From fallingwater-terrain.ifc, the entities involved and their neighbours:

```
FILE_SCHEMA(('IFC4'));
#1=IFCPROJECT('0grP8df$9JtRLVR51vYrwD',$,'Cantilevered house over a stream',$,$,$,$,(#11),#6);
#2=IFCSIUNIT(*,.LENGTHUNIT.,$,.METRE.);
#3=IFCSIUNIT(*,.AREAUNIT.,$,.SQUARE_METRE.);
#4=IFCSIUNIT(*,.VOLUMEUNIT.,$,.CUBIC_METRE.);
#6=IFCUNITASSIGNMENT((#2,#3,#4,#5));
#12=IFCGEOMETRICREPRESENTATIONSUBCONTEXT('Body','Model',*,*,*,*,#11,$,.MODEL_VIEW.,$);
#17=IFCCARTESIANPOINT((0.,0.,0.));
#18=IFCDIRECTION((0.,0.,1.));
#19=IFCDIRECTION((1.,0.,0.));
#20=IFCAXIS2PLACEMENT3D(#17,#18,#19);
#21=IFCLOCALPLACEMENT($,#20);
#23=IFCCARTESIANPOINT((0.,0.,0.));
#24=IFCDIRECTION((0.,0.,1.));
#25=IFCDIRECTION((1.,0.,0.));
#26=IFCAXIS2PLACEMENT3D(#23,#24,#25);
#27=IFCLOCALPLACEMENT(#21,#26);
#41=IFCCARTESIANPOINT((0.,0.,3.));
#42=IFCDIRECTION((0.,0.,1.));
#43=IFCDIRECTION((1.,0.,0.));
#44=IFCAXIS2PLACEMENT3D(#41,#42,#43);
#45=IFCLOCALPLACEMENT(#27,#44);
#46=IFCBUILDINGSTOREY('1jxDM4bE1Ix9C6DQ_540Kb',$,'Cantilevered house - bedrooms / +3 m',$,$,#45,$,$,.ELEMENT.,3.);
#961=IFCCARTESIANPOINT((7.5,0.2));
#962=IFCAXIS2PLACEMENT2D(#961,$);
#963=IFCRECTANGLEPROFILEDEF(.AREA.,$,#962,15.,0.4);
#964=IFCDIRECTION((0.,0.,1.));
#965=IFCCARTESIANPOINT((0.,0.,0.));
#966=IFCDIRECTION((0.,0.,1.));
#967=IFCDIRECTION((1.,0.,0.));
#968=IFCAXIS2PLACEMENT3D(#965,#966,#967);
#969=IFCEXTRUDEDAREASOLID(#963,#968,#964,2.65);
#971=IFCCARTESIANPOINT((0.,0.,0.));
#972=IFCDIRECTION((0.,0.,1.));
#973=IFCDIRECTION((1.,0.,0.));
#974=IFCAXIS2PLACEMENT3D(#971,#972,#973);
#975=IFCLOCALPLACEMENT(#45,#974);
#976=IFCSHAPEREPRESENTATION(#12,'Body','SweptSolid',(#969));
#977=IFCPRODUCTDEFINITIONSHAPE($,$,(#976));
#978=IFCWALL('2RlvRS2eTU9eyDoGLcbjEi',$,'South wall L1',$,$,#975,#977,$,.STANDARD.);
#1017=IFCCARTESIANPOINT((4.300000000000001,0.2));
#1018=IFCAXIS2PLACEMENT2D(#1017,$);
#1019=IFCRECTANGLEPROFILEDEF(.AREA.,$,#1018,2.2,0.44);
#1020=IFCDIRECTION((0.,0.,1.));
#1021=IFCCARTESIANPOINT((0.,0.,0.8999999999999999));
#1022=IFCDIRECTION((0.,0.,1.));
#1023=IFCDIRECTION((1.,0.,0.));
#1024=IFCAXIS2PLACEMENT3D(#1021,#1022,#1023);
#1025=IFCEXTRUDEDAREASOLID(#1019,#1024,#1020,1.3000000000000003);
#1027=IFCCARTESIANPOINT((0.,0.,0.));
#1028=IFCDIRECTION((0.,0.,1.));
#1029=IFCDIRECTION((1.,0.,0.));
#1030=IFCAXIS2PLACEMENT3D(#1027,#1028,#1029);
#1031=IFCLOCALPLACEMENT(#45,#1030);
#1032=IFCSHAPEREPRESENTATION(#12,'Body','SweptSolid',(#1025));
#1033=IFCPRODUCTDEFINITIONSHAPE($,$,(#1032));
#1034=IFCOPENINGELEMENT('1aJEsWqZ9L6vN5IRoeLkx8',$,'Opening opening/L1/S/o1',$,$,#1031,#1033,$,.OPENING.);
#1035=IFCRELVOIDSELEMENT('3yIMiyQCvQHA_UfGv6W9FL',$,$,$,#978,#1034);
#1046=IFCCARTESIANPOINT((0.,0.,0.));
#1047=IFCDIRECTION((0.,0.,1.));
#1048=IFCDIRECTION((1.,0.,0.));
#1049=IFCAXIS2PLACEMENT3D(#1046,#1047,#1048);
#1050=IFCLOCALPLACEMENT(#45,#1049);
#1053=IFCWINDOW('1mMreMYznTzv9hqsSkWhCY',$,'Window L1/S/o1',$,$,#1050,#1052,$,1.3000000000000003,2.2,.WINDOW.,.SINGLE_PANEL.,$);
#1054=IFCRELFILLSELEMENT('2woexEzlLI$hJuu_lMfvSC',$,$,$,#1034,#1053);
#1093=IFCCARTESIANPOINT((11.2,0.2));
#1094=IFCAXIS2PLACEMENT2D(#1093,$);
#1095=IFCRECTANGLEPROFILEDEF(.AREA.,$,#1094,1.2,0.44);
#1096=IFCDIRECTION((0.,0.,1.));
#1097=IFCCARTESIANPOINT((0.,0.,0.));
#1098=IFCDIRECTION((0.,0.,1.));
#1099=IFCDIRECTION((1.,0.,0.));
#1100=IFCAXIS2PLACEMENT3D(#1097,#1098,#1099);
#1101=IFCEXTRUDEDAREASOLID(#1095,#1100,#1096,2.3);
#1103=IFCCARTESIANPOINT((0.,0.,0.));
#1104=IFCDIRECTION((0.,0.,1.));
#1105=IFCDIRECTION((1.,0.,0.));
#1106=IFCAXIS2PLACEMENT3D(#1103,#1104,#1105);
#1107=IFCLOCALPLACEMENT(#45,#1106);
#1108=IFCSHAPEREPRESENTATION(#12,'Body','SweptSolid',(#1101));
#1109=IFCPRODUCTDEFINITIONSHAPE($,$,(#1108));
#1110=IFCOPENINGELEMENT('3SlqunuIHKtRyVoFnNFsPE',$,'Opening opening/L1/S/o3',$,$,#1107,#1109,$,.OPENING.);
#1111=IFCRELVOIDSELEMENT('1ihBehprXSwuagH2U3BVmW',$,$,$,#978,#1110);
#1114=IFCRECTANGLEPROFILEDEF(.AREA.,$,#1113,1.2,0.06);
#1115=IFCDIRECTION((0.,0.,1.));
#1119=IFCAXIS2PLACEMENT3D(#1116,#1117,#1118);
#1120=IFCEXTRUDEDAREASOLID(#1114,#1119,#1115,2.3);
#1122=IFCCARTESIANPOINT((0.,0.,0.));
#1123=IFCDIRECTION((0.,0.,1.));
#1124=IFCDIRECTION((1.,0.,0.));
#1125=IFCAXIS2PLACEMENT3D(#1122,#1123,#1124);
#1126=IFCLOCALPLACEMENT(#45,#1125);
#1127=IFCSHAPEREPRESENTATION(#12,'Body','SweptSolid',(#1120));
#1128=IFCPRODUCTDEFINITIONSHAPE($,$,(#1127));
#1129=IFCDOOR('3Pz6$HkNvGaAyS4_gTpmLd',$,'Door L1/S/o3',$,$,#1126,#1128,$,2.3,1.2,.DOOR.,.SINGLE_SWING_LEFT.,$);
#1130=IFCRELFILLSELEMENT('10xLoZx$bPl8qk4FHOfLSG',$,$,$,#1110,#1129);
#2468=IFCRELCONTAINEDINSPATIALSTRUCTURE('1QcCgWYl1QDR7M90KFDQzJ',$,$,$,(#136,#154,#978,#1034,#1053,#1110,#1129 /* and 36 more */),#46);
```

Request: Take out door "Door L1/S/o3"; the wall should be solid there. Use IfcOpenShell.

```python
import ifcopenshell
import ifcopenshell.api.feature
import ifcopenshell.api.root
import ifcopenshell.geom
import ifcopenshell.util.shape

model = ifcopenshell.open("fallingwater-terrain.ifc")
settings = ifcopenshell.geom.settings()


def volume(element):
    """Net volume in cubic metres, openings subtracted."""
    shape = ifcopenshell.geom.create_shape(settings, element)
    return ifcopenshell.util.shape.get_volume(shape.geometry)


door = model.by_guid("3Pz6$HkNvGaAyS4_gTpmLd")
opening = door.FillsVoids[0].RelatingOpeningElement
wall = opening.VoidsElements[0].RelatingBuildingElement
before = volume(wall)

ifcopenshell.api.root.remove_product(model, product=door)
ifcopenshell.api.feature.remove_feature(model, feature=opening)

after = volume(wall)

print(f"wall volume {before:.3f} -> {after:.3f} m3")

model.write("fallingwater-terrain_rev.ifc")
```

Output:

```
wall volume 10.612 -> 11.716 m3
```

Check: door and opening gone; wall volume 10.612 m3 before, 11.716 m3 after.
